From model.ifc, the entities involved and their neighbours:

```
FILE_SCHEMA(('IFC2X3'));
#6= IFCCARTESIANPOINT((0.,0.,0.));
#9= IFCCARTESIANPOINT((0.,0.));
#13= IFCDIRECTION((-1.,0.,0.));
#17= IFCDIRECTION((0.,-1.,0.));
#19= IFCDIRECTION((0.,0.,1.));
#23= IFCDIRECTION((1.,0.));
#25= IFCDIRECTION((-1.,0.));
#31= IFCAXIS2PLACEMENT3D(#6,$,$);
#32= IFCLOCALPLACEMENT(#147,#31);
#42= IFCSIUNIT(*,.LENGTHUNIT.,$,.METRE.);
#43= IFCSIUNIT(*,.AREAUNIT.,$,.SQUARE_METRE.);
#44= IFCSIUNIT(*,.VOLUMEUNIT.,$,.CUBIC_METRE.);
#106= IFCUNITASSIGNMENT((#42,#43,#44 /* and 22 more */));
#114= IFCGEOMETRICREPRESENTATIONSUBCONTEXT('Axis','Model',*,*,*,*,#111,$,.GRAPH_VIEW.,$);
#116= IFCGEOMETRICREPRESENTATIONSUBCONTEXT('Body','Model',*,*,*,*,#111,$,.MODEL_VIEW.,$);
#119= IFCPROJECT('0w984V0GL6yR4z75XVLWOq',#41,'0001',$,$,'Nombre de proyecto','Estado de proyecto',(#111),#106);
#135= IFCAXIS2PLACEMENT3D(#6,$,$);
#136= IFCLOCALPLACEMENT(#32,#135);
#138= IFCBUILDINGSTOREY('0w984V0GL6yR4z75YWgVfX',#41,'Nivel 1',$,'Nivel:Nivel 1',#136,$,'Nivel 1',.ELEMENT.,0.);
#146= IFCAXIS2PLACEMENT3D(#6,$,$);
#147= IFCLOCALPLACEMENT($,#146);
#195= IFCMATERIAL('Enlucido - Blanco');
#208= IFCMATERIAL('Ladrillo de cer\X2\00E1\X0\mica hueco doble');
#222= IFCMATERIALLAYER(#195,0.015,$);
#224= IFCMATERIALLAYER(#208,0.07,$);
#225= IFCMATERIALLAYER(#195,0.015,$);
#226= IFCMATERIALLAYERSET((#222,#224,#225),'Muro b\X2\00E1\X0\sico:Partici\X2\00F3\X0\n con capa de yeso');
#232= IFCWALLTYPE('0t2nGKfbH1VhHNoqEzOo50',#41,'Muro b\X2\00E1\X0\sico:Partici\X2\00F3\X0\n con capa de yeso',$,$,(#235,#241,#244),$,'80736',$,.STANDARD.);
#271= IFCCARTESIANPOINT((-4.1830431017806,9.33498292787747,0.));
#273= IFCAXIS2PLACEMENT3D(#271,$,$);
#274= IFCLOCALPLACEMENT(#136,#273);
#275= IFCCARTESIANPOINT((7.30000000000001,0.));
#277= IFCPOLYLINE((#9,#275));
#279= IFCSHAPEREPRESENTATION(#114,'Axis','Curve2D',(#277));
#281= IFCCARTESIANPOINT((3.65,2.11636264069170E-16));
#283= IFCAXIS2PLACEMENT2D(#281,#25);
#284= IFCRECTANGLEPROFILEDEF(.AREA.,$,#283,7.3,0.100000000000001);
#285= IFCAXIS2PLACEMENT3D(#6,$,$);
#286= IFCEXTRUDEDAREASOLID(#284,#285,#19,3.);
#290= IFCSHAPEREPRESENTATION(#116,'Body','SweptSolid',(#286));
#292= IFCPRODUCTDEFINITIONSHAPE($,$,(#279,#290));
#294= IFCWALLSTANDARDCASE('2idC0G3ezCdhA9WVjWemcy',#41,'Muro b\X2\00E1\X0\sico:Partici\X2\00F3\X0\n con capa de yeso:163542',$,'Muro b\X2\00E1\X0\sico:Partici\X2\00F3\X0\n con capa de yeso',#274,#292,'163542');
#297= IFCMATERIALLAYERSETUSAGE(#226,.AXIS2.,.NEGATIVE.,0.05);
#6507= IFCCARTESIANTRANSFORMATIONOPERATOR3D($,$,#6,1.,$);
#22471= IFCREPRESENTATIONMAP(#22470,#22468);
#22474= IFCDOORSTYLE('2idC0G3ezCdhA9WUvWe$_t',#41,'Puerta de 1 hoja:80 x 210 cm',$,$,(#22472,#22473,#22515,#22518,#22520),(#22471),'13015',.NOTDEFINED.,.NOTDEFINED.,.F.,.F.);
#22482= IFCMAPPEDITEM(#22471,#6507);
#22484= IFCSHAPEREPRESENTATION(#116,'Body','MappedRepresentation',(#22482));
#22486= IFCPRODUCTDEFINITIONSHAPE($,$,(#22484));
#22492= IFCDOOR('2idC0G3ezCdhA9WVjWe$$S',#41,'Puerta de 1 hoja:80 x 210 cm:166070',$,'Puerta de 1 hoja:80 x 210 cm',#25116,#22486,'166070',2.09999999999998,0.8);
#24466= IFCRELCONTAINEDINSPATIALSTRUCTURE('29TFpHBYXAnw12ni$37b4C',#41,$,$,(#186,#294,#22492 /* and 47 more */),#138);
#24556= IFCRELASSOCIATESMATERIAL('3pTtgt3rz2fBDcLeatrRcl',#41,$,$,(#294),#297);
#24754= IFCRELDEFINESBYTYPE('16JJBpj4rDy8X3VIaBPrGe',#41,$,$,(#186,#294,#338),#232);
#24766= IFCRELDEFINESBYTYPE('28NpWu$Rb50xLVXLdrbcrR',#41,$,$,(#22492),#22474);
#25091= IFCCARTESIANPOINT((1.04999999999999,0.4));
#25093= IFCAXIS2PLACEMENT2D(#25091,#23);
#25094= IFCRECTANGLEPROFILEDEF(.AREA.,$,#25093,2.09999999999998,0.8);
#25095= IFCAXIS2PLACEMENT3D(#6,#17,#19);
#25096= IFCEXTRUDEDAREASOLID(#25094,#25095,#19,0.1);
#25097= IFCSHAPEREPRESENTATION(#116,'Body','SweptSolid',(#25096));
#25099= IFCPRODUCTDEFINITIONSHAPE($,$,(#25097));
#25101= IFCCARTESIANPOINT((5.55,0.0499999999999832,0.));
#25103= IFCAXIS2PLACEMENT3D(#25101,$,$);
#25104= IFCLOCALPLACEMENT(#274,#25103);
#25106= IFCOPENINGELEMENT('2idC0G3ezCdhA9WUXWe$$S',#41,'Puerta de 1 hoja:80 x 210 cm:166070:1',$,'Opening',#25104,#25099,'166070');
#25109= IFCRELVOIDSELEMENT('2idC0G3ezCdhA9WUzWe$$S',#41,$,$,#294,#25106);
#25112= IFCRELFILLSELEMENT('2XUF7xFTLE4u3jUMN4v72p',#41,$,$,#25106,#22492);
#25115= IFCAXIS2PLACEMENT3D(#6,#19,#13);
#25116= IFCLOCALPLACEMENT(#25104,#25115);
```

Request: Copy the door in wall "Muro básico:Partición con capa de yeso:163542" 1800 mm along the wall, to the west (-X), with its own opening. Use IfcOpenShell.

```python
import ifcopenshell
import ifcopenshell.api.feature
import ifcopenshell.api.geometry
import ifcopenshell.api.root
import ifcopenshell.geom
import ifcopenshell.util.element
import ifcopenshell.util.placement
import ifcopenshell.util.shape
import ifcopenshell.util.unit

model = ifcopenshell.open("model.ifc")
unit_scale = ifcopenshell.util.unit.calculate_unit_scale(model)
settings = ifcopenshell.geom.settings()


def volume(element):
    """Net volume in cubic metres, openings subtracted."""
    shape = ifcopenshell.geom.create_shape(settings, element)
    return ifcopenshell.util.shape.get_volume(shape.geometry)


def reuse_history(source, copy):
    """copy_class also copies each property set's owner history, people and application; keep the originals."""
    for rel in copy.IsDefinedBy:
        if rel.is_a("IfcRelDefinesByProperties") and (history := rel.RelatingPropertyDefinition.OwnerHistory):
            rel.RelatingPropertyDefinition.OwnerHistory = source.OwnerHistory
            ifcopenshell.util.element.remove_deep2(model, history)


door = model.by_guid("2idC0G3ezCdhA9WVjWe$$S")
opening = door.FillsVoids[0].RelatingOpeningElement
wall = opening.VoidsElements[0].RelatingBuildingElement
before = volume(wall)
shift = ifcopenshell.util.placement.get_local_placement(wall.ObjectPlacement)[:3, 0] * -1.8 / unit_scale

# copy_class copies the void relationship, type, container and properties, but no geometry.
new_opening = ifcopenshell.api.root.copy_class(model, product=opening)
new_opening.Representation = ifcopenshell.util.element.copy_deep(
    model, opening.Representation, exclude=["IfcGeometricRepresentationContext", "IfcRepresentationMap"]
)
new_opening.Name = "Puerta de 1 hoja:80 x 210 cm"
new_opening.Tag = None
new_door = ifcopenshell.api.root.copy_class(model, product=door)
new_door.Representation = ifcopenshell.util.element.copy_deep(
    model, door.Representation, exclude=["IfcGeometricRepresentationContext", "IfcRepresentationMap"]
)
new_door.Name = "Puerta de 1 hoja:80 x 210 cm"
new_door.Tag = None
reuse_history(door, new_door)
fills = ifcopenshell.api.feature.add_filling(model, opening=new_opening, element=new_door)
fills.OwnerHistory = new_door.OwnerHistory  # required in IFC2X3

for old, new in ((opening, new_opening), (door, new_door)):
    matrix = ifcopenshell.util.placement.get_local_placement(old.ObjectPlacement)
    matrix[:3, 3] += shift
    ifcopenshell.api.geometry.edit_object_placement(model, product=new, matrix=matrix, is_si=False)

after = volume(wall)

print(f"wall volume {before:.3f} -> {after:.3f} m3")

model.write("model_updated.ifc")
```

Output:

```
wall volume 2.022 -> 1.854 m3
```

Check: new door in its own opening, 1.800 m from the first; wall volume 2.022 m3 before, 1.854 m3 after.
